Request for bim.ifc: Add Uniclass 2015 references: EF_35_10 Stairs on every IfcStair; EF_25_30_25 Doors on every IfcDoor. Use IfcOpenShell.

First a look at what the model holds.

```python
import ifcopenshell

model = ifcopenshell.open("bim.ifc")
print(model.schema)
print("classifications:", [c.Name for c in model.by_type("IfcClassification")])
for ifc_class in ("IfcDoor", "IfcRoof", "IfcStair", "IfcWall", "IfcWindow"):
    print(ifc_class, len(model.by_type(ifc_class)))
```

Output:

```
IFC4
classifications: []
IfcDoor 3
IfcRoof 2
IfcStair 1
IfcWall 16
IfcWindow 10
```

```python
import ifcopenshell
import ifcopenshell.api.classification

model = ifcopenshell.open("bim.ifc")

system = ifcopenshell.api.classification.add_classification(model, classification="Uniclass 2015")

codes = {
    "IfcStair": ("EF_35_10", "Stairs"),
    "IfcDoor": ("EF_25_30_25", "Doors"),
}
for ifc_class, (code, name) in codes.items():
    products = model.by_type(ifc_class)
    ifcopenshell.api.classification.add_reference(
        model, products=products, classification=system, identification=code, name=name
    )
    print(code, len(products))

model.write("bim_edited.ifc")
```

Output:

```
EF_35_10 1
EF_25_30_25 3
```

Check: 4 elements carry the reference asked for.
